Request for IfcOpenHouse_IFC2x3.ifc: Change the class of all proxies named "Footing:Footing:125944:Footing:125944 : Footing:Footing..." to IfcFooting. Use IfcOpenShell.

First a look at what the model holds.

```python
import re

import ifcopenshell

model = ifcopenshell.open("IfcOpenHouse_IFC2x3.ifc")
print(model.schema)
seen = {}
for e in model.by_type("IfcBuildingElementProxy"):
    name = re.sub(r":\d+(:\d+)?$", "", e.Name or "")  # drop the element id that some exporters append
    seen[name] = seen.get(name, 0) + 1
for name, count in sorted(seen.items()):
    print(count, "x", name)
```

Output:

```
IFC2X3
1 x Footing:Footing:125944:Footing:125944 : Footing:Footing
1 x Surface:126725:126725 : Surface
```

```python
import ifcopenshell
import ifcopenshell.api.root

model = ifcopenshell.open("IfcOpenHouse_IFC2x3.ifc")

proxies = [e.id() for e in model.by_type("IfcBuildingElementProxy") if (e.Name or "").startswith("Footing:Footing:125944:Footing:125944 : Footing:Footing")]
for step_id in proxies:
    proxy = model.by_id(step_id)
    ifcopenshell.api.root.reassign_class(model, product=proxy, ifc_class="IfcFooting", predefined_type="NOTDEFINED")

print(sum(model.by_id(i).is_a("IfcFooting") for i in proxies), "reclassified")

model.write("IfcOpenHouse_IFC2x3_edited.ifc")
```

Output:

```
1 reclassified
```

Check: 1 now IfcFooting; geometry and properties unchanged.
